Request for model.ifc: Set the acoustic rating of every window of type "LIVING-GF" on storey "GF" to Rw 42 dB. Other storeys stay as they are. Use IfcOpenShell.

First a look at what the model holds.

```python
import ifcopenshell
import ifcopenshell.util.element

model = ifcopenshell.open("model.ifc")
print(model.schema)
storey = next(s for s in model.by_type("IfcBuildingStorey") if s.Name == "GF")
windows = [e for e in ifcopenshell.util.element.get_decomposition(storey) if e.is_a("IfcWindow")]
seen = {}
for e in windows:
    element_type = ifcopenshell.util.element.get_type(e)
    key = (element_type.Name if element_type != e and element_type else None, ifcopenshell.util.element.get_pset(e, "Pset_WindowCommon", "AcousticRating"))
    seen[key] = seen.get(key, 0) + 1
for (name, value), count in sorted(seen.items(), key=str):
    print(count, "x", name, "|", value)
```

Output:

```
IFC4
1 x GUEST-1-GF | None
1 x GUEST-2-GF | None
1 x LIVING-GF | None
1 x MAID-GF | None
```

```python
import ifcopenshell
import ifcopenshell.api.pset
import ifcopenshell.util.element

model = ifcopenshell.open("model.ifc")

storey = next(s for s in model.by_type("IfcBuildingStorey") if s.Name == "GF")
windows = [e for e in ifcopenshell.util.element.get_decomposition(storey) if e.is_a("IfcWindow")]

count = 0
for e in windows:
    element_type = ifcopenshell.util.element.get_type(e)
    if element_type in (None, e) or element_type.Name != "LIVING-GF":
        continue
    # add_pset returns the element's existing set when there is one.
    pset = ifcopenshell.api.pset.add_pset(model, product=e, name="Pset_WindowCommon")
    ifcopenshell.api.pset.edit_pset(model, pset=pset, properties={"AcousticRating": "Rw 42 dB"})
    count += 1

print(count, "windows updated")

model.write("model_edited.ifc")
```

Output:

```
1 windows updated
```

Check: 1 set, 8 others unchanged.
